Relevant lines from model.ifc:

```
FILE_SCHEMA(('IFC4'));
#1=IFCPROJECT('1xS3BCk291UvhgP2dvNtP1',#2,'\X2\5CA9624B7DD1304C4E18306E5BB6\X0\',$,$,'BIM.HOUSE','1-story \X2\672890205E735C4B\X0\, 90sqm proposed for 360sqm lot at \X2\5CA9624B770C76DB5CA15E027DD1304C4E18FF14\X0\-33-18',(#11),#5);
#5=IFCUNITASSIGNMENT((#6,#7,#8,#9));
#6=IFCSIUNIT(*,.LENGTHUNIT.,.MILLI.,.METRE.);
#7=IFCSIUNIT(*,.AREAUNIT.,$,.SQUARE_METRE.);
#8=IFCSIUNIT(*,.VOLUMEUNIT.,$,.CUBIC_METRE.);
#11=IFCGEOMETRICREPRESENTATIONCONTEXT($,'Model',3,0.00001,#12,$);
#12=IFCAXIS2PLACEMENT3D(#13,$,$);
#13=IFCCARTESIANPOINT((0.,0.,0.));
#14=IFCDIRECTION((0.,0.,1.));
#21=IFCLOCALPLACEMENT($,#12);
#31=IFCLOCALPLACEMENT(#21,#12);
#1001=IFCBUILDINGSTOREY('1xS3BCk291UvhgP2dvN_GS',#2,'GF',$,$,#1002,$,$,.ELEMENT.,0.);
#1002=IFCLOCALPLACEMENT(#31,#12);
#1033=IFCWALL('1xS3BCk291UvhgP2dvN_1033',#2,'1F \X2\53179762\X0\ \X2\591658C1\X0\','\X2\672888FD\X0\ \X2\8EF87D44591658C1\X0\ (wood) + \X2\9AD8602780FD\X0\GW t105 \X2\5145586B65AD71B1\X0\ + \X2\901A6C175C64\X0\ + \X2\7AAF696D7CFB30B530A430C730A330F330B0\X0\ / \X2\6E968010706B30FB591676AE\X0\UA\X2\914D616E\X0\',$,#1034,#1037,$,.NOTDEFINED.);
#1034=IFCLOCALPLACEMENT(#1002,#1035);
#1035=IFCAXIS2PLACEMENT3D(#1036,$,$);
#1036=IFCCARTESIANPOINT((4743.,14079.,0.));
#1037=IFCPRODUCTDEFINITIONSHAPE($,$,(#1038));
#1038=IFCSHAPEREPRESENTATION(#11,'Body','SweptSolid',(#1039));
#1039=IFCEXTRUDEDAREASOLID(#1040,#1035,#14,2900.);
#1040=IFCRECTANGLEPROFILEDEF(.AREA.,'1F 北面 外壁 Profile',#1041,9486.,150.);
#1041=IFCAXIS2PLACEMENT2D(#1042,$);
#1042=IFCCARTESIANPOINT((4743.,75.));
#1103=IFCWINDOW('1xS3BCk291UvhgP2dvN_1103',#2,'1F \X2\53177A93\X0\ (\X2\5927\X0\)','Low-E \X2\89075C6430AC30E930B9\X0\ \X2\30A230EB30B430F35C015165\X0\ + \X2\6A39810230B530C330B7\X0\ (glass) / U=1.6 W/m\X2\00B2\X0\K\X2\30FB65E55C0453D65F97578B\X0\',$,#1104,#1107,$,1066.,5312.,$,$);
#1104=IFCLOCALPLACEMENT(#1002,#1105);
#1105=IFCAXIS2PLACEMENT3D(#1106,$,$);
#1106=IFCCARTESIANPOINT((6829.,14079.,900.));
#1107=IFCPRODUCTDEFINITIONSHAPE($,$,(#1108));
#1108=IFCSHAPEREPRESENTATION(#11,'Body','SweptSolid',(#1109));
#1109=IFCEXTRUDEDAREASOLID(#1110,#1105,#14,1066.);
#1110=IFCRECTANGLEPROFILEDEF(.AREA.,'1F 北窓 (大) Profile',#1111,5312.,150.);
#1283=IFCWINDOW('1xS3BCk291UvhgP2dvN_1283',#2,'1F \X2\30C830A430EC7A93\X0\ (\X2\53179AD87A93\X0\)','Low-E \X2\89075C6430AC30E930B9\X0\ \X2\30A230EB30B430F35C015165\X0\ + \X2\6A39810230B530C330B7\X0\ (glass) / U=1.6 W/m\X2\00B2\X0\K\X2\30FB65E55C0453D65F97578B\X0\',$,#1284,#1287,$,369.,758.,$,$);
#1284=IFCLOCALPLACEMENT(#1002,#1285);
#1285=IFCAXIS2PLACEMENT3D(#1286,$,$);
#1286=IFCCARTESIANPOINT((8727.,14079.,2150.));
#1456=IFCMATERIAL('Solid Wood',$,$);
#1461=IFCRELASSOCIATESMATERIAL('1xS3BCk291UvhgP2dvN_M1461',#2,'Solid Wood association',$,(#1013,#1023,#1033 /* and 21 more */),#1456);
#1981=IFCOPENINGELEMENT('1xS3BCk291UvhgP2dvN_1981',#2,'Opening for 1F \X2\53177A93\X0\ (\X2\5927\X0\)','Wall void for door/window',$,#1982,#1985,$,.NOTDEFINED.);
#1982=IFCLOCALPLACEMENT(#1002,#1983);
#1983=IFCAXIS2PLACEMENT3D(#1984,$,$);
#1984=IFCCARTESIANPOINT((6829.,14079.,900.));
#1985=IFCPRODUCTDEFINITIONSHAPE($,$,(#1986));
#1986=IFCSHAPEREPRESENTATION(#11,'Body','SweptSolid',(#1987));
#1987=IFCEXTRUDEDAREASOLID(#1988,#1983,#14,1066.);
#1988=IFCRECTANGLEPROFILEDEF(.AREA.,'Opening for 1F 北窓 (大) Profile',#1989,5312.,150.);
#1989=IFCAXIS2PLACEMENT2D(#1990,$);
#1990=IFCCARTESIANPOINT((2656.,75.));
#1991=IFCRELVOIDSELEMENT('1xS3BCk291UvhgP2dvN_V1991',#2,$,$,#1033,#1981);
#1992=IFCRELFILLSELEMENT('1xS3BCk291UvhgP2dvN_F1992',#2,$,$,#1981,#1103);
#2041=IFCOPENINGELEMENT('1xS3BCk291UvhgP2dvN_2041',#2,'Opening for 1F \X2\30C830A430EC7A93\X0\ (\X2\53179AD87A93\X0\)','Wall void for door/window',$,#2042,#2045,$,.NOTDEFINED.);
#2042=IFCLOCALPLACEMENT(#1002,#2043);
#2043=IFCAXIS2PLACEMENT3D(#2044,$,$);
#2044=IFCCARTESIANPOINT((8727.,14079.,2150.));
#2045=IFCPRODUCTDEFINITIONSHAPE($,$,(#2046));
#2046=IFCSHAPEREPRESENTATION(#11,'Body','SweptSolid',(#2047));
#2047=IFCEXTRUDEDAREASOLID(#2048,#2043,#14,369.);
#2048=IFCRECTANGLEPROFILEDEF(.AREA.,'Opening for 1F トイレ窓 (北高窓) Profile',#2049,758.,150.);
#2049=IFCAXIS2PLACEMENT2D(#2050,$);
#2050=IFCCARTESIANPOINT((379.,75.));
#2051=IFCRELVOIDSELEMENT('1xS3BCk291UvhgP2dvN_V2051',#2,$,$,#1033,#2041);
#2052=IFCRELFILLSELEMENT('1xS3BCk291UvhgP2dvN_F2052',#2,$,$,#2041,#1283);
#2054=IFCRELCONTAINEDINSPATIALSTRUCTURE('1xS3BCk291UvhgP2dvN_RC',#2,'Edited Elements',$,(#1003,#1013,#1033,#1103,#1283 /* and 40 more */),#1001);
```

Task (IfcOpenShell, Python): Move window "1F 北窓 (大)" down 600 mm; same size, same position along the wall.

```python
import numpy as np
import ifcopenshell
import ifcopenshell.api.geometry
import ifcopenshell.util.placement
import ifcopenshell.util.unit

model = ifcopenshell.open("model.ifc")
unit_scale = ifcopenshell.util.unit.calculate_unit_scale(model)

window = model.by_guid("1xS3BCk291UvhgP2dvN_1103")
opening = window.FillsVoids[0].RelatingOpeningElement
dz = -0.6 / unit_scale

shift = np.array([0.0, 0.0, dz])
# The window is not placed relative to its opening, so move both.
for product in (opening, window):
    matrix = ifcopenshell.util.placement.get_local_placement(product.ObjectPlacement)
    matrix[:3, 3] += shift
    ifcopenshell.api.geometry.edit_object_placement(model, product=product, matrix=matrix, is_si=False)

print(f"moved by {dz * unit_scale:+.3f} m")

model.write("model_updated.ifc")
```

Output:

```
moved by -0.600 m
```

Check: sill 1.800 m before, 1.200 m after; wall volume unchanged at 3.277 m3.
